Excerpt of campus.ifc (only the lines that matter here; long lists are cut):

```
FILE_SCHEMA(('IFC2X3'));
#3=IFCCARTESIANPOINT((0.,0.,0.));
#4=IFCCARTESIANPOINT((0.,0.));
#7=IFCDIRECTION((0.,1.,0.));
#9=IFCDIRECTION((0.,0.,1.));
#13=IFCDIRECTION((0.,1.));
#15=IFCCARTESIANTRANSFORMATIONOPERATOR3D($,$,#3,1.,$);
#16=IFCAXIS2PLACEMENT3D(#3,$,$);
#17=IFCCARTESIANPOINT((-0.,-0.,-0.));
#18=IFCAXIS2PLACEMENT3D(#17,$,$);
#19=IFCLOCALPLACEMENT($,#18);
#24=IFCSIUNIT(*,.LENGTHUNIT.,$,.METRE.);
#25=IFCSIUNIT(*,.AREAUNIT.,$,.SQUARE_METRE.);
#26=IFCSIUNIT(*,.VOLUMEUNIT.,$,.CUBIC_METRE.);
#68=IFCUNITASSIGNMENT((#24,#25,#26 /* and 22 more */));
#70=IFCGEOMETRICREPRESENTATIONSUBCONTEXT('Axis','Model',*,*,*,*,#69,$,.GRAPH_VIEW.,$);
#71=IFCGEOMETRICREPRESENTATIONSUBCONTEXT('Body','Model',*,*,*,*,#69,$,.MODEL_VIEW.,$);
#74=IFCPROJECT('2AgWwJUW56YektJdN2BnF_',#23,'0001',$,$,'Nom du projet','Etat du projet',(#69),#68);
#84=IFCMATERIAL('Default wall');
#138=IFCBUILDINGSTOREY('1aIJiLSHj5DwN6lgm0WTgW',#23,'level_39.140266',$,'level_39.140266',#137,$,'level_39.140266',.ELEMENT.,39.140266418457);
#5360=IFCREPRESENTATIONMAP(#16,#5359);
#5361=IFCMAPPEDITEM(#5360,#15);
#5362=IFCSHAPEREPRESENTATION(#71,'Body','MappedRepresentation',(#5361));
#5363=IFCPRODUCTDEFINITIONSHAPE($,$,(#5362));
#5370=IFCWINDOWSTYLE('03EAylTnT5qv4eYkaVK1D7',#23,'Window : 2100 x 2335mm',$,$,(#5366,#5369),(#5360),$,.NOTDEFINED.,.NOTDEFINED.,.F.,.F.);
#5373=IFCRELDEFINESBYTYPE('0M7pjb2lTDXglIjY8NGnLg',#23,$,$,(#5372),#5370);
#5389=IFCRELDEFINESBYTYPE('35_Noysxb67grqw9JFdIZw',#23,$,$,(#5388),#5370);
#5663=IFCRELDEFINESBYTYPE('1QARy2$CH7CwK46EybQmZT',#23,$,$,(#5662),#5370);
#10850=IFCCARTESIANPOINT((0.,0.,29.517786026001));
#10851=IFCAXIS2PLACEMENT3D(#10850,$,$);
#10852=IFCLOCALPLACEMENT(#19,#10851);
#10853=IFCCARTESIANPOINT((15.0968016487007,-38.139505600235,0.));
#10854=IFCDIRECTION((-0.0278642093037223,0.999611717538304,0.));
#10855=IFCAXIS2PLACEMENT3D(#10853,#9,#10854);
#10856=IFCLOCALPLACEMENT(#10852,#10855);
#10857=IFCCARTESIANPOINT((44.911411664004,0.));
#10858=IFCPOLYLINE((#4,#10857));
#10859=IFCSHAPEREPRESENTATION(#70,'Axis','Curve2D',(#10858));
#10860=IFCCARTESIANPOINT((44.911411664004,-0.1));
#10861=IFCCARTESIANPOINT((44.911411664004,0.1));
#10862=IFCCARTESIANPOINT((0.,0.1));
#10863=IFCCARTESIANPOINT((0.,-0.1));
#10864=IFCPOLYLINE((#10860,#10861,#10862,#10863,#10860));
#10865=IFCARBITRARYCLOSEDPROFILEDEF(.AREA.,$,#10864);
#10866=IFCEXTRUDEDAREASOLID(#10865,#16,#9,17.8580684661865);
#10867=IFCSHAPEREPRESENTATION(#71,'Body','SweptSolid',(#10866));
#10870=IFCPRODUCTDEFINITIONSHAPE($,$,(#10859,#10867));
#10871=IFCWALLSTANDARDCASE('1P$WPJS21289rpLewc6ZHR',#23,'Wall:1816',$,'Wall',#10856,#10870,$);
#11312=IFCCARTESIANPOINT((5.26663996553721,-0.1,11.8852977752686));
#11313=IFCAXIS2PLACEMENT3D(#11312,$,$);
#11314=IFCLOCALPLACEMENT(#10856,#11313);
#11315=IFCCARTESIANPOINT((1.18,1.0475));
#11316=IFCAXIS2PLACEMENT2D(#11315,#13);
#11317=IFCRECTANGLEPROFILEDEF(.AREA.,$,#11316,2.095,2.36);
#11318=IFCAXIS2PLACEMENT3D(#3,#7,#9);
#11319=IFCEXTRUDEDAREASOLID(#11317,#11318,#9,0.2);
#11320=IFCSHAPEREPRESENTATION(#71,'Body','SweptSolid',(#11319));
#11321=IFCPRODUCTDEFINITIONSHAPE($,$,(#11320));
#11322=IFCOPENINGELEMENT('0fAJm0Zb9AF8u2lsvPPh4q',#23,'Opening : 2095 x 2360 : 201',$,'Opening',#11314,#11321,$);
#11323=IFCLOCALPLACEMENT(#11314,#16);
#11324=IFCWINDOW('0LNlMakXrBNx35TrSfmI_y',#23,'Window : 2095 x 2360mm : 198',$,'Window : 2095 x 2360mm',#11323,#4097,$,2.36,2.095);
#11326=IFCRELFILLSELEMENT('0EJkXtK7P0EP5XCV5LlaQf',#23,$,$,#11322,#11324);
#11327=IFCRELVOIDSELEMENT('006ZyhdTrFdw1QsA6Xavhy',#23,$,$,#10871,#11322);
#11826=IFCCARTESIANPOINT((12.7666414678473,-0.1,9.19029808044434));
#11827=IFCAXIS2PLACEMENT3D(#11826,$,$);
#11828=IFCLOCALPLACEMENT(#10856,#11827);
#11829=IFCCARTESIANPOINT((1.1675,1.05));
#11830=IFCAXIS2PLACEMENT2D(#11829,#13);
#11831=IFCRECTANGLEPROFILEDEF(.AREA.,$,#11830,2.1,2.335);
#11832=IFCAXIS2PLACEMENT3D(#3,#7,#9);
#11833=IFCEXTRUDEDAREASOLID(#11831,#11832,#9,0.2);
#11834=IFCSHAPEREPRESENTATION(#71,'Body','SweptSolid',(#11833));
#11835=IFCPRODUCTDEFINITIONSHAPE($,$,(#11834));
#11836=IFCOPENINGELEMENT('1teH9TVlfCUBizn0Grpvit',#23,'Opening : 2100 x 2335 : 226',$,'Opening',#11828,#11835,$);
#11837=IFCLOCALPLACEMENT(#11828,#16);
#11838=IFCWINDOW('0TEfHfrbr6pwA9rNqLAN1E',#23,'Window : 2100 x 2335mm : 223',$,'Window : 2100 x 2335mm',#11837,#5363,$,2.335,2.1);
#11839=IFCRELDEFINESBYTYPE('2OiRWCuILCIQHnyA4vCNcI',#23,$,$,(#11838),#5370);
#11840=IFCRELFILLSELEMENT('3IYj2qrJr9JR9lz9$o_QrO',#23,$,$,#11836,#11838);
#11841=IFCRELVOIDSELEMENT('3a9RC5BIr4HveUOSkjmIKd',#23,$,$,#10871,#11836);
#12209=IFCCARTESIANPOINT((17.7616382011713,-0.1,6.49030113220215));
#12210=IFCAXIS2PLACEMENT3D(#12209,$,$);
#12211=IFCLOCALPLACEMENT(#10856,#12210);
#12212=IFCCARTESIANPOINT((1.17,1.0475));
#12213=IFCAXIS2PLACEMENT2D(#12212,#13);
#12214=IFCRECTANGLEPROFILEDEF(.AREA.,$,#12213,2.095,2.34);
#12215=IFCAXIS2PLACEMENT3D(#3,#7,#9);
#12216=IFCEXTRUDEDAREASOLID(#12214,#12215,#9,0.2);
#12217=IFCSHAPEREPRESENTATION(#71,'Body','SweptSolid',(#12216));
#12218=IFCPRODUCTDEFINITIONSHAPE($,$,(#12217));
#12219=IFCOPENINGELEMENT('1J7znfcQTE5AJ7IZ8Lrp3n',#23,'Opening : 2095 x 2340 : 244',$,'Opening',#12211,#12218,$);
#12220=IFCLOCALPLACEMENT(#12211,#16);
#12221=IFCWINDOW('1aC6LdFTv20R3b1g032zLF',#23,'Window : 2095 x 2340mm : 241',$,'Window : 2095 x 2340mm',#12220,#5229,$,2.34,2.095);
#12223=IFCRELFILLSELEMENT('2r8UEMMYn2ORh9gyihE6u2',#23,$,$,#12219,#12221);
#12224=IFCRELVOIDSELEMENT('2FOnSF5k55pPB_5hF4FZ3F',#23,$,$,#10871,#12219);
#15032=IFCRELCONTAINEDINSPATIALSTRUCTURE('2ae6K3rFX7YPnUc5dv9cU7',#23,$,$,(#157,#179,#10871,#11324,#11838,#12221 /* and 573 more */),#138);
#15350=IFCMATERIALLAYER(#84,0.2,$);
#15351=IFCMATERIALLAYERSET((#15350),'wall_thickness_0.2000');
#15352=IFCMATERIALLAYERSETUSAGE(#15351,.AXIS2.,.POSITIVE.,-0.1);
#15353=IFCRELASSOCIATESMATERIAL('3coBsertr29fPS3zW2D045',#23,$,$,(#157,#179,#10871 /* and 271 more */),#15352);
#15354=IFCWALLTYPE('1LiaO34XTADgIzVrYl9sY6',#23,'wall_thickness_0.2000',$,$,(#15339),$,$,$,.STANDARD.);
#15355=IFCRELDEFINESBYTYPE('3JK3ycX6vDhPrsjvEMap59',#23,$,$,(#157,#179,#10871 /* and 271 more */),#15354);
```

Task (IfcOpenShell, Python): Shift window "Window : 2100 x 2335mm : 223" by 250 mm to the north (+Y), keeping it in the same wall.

```python
import ifcopenshell
import ifcopenshell.api.geometry
import ifcopenshell.util.placement
import ifcopenshell.util.unit

model = ifcopenshell.open("campus.ifc")
unit_scale = ifcopenshell.util.unit.calculate_unit_scale(model)

window = model.by_id(11838)
opening = window.FillsVoids[0].RelatingOpeningElement
wall = opening.VoidsElements[0].RelatingBuildingElement

wall_matrix = ifcopenshell.util.placement.get_local_placement(wall.ObjectPlacement)
shift = wall_matrix[:3, 0] * 0.25 / unit_scale
before = ifcopenshell.util.placement.get_local_placement(window.ObjectPlacement)[:3, 3].copy()

# The window is placed relative to its opening, so it follows when the opening moves.
matrix = ifcopenshell.util.placement.get_local_placement(opening.ObjectPlacement)
matrix[:3, 3] += shift
ifcopenshell.api.geometry.edit_object_placement(
    model, product=opening, matrix=matrix, is_si=False, should_transform_children=True
)

after = ifcopenshell.util.placement.get_local_placement(window.ObjectPlacement)[:3, 3]
print("window moved by", (after - before).round(3) + 0.0)

model.write("campus_updated.ifc")
```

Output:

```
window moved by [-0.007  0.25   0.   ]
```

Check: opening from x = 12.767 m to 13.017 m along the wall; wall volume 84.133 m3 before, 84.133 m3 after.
